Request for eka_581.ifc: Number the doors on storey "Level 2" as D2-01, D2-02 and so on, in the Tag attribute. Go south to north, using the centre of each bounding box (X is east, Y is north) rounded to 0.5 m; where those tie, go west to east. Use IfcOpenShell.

First a look at what the model holds.

```python
import ifcopenshell
import ifcopenshell.util.element
import ifcopenshell.util.placement

model = ifcopenshell.open("eka_581.ifc")
print(model.schema)
storey = next(s for s in model.by_type("IfcBuildingStorey") if s.Name == "Level 2")
doors = [e for e in ifcopenshell.util.element.get_decomposition(storey) if e.is_a("IfcDoor")]
for e in sorted(doors, key=lambda e: e.id()):
    origin = ifcopenshell.util.placement.get_local_placement(e.ObjectPlacement)[:3, 3]
    print(e.id(), e.Tag, e.Name, origin.round(2) + 0.0, sep=" | ")
```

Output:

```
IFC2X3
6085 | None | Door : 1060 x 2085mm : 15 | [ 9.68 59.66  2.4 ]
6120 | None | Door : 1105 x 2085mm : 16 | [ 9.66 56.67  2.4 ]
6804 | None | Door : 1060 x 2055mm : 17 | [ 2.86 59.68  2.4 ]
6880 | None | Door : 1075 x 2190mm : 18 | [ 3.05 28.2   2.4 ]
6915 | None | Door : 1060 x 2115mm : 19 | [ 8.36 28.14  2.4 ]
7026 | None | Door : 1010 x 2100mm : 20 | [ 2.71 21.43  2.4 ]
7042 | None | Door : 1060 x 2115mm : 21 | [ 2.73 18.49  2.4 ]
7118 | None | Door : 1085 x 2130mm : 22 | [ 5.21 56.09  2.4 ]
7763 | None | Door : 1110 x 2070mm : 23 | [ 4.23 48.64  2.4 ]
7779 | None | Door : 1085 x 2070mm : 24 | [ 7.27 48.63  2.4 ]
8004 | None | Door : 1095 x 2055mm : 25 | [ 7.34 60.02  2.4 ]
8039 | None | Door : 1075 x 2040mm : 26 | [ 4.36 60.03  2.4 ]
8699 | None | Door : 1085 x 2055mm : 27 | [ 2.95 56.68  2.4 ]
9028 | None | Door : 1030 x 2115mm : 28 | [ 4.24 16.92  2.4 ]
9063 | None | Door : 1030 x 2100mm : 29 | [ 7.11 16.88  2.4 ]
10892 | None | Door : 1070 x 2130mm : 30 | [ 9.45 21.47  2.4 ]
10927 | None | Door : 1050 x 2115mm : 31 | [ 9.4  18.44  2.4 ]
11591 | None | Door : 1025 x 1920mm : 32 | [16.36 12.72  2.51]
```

```python
import ifcopenshell
import ifcopenshell.geom
import ifcopenshell.util.element
import ifcopenshell.util.shape

model = ifcopenshell.open("eka_581.ifc")
settings = ifcopenshell.geom.settings()
settings.set("use-world-coords", True)


def centre(element):
    shape = ifcopenshell.geom.create_shape(settings, element)
    return ifcopenshell.util.shape.get_bbox_centroid(shape.geometry)


storey = next(s for s in model.by_type("IfcBuildingStorey") if s.Name == "Level 2")
doors = [e for e in ifcopenshell.util.element.get_decomposition(storey) if e.is_a("IfcDoor")]

# Insertion points can sit at a corner or the storey origin, so sort by the geometry (in metres).
centres = {e: centre(e) for e in doors}
doors.sort(key=lambda e: (round(centres[e][1] / 0.5), centres[e][0]))

for i, e in enumerate(doors, start=1):
    number = f"D2-{i:02d}"
    e.Tag = number
    print(e.id(), number)

model.write("eka_581-out.ifc")
```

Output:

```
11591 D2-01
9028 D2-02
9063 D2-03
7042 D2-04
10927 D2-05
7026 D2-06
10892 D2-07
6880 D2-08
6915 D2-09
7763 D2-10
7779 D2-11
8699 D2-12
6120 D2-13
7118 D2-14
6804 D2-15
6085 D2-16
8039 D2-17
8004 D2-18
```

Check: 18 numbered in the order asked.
